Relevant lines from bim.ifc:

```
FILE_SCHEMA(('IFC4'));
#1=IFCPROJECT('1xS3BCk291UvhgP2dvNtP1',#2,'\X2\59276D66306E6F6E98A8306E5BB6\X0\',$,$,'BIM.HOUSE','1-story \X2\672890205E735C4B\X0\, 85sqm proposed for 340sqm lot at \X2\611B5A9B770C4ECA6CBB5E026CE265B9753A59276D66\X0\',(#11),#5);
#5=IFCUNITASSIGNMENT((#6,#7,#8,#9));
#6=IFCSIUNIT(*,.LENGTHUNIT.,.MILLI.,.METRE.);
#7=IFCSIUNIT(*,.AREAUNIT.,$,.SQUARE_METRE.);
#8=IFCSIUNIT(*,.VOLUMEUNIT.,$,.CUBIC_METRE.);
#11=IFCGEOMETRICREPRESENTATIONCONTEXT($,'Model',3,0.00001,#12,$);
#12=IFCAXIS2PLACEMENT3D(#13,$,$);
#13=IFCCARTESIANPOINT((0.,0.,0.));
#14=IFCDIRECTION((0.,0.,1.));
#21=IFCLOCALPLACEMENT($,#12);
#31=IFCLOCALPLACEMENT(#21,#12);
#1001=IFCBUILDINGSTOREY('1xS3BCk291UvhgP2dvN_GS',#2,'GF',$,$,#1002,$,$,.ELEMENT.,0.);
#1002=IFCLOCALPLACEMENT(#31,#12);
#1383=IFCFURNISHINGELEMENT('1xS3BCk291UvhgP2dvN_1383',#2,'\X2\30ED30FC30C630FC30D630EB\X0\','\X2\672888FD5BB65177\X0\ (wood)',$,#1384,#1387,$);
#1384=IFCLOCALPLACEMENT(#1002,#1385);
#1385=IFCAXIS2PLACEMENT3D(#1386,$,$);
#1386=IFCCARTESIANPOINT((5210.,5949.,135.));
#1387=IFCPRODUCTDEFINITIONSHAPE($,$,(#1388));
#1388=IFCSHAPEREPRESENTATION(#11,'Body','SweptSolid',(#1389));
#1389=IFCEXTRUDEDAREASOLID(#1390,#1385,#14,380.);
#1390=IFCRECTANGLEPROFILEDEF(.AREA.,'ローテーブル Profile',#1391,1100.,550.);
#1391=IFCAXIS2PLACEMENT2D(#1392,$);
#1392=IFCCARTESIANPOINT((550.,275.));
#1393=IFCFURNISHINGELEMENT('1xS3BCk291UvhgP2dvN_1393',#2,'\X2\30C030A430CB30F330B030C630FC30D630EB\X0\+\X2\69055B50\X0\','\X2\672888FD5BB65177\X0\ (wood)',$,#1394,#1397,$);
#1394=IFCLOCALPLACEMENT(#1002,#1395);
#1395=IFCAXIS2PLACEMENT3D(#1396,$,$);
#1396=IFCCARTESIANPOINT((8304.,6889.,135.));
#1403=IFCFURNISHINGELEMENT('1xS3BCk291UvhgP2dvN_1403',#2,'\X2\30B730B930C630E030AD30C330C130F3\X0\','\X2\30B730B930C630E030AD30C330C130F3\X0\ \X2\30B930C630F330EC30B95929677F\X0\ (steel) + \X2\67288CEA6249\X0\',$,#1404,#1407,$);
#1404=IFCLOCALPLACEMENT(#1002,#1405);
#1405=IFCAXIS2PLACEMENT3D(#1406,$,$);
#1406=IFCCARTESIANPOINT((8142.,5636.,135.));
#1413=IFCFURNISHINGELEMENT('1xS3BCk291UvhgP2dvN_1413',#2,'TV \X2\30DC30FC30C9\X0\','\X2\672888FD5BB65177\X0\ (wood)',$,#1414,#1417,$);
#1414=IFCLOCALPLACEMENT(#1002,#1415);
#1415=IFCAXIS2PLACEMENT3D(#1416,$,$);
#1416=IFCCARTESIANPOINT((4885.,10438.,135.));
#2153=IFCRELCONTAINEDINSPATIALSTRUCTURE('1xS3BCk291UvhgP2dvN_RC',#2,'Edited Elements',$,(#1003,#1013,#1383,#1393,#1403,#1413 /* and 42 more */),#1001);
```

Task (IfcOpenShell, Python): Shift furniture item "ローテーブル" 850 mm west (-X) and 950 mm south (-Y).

```python
import ifcopenshell
import ifcopenshell.api.geometry
import ifcopenshell.util.placement
import ifcopenshell.util.unit

model = ifcopenshell.open("bim.ifc")
unit_scale = ifcopenshell.util.unit.calculate_unit_scale(model)

item = model.by_guid("1xS3BCk291UvhgP2dvN_1383")
matrix = ifcopenshell.util.placement.get_local_placement(item.ObjectPlacement)
matrix[0, 3] -= 0.85 / unit_scale
matrix[1, 3] -= 0.95 / unit_scale
ifcopenshell.api.geometry.edit_object_placement(model, product=item, matrix=matrix, is_si=False)

print(ifcopenshell.util.placement.get_local_placement(item.ObjectPlacement).round(3) + 0.0)

model.write("bim_v2.ifc")
```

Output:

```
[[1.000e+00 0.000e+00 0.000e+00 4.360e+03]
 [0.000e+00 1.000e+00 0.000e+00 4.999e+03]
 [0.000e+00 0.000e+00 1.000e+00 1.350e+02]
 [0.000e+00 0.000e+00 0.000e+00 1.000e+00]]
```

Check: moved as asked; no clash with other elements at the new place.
